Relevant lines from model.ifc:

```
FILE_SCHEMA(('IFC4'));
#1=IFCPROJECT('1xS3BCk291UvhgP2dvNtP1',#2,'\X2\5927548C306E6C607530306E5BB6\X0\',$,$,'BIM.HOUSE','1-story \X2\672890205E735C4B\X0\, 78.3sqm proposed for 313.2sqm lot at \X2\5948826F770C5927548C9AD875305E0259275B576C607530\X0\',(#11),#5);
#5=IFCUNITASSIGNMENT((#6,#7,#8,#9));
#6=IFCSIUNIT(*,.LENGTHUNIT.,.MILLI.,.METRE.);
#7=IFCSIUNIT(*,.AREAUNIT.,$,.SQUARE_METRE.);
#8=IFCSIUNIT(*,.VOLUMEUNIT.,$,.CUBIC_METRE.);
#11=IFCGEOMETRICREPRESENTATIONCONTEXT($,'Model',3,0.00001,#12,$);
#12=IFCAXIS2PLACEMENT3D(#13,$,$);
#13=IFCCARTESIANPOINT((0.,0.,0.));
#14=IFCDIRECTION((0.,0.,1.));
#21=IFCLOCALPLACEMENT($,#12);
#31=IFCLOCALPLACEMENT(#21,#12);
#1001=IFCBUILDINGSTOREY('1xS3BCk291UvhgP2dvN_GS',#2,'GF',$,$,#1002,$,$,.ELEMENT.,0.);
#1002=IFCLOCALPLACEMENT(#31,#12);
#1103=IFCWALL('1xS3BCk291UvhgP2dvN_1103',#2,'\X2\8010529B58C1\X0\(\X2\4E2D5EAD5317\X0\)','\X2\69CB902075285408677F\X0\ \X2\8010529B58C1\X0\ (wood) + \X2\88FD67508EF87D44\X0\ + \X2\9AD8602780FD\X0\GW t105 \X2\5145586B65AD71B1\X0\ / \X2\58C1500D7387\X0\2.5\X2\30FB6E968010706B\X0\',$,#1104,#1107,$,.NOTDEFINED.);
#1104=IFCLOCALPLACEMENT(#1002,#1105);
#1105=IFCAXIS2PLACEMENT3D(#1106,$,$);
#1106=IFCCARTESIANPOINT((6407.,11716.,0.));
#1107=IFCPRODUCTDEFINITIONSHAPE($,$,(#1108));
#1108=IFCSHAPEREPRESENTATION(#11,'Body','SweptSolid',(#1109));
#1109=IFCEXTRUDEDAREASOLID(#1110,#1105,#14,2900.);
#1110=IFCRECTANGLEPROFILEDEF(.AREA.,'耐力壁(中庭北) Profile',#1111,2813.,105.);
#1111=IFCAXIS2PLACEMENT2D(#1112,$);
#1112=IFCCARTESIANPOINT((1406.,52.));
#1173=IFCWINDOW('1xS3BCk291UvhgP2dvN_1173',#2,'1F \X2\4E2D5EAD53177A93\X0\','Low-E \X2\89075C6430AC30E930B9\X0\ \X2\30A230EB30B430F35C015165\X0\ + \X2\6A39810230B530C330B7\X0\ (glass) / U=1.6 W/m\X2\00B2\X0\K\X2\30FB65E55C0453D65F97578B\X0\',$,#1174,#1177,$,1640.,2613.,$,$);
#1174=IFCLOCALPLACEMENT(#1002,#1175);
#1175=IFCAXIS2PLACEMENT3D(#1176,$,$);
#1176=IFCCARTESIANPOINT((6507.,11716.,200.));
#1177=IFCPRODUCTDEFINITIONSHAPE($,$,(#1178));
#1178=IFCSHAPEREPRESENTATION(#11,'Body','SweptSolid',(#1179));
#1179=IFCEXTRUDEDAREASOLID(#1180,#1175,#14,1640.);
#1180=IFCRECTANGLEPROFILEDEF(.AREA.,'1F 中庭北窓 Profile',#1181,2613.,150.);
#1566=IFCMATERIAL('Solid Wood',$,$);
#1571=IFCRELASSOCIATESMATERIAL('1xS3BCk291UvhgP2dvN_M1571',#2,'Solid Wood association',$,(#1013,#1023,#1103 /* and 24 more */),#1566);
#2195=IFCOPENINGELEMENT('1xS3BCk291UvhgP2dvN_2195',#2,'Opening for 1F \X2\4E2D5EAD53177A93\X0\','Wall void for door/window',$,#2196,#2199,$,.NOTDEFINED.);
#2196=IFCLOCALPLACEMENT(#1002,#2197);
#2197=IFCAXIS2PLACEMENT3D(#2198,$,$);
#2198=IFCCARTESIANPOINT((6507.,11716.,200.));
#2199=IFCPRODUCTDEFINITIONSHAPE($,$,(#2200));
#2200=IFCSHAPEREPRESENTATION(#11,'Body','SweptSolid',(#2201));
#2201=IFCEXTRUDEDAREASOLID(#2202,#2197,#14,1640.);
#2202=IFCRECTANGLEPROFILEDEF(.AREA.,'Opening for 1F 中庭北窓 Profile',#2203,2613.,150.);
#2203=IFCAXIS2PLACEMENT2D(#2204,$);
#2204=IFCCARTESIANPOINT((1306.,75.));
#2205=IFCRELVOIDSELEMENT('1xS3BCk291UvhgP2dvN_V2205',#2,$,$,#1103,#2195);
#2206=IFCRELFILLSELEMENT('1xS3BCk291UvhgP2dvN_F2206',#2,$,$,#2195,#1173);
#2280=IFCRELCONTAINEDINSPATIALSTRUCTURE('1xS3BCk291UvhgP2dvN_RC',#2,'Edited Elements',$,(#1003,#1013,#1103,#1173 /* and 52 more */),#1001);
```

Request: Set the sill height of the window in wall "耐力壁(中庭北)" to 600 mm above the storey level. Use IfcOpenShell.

```python
import numpy as np
import ifcopenshell
import ifcopenshell.api.geometry
import ifcopenshell.geom
import ifcopenshell.util.element
import ifcopenshell.util.placement
import ifcopenshell.util.shape
import ifcopenshell.util.unit

model = ifcopenshell.open("model.ifc")
unit_scale = ifcopenshell.util.unit.calculate_unit_scale(model)

window = model.by_guid("1xS3BCk291UvhgP2dvN_1173")
opening = window.FillsVoids[0].RelatingOpeningElement
storey = ifcopenshell.util.element.get_container(window, ifc_class="IfcBuildingStorey")
level = ifcopenshell.util.placement.get_local_placement(storey.ObjectPlacement)[2, 3]

# The opening's origin need not be at the sill, so measure its lowest point.
shape = ifcopenshell.geom.create_shape(ifcopenshell.geom.settings(), opening)
bottom = ifcopenshell.util.shape.get_shape_bottom_elevation(shape, shape.geometry) / unit_scale
dz = level + 0.6 / unit_scale - bottom

shift = np.array([0.0, 0.0, dz])
# The window is not placed relative to its opening, so move both.
for product in (opening, window):
    matrix = ifcopenshell.util.placement.get_local_placement(product.ObjectPlacement)
    matrix[:3, 3] += shift
    ifcopenshell.api.geometry.edit_object_placement(model, product=product, matrix=matrix, is_si=False)

print(f"moved by {dz * unit_scale:+.3f} m")

model.write("model_rev.ifc")
```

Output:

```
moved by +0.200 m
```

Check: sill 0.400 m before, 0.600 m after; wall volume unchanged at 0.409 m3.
